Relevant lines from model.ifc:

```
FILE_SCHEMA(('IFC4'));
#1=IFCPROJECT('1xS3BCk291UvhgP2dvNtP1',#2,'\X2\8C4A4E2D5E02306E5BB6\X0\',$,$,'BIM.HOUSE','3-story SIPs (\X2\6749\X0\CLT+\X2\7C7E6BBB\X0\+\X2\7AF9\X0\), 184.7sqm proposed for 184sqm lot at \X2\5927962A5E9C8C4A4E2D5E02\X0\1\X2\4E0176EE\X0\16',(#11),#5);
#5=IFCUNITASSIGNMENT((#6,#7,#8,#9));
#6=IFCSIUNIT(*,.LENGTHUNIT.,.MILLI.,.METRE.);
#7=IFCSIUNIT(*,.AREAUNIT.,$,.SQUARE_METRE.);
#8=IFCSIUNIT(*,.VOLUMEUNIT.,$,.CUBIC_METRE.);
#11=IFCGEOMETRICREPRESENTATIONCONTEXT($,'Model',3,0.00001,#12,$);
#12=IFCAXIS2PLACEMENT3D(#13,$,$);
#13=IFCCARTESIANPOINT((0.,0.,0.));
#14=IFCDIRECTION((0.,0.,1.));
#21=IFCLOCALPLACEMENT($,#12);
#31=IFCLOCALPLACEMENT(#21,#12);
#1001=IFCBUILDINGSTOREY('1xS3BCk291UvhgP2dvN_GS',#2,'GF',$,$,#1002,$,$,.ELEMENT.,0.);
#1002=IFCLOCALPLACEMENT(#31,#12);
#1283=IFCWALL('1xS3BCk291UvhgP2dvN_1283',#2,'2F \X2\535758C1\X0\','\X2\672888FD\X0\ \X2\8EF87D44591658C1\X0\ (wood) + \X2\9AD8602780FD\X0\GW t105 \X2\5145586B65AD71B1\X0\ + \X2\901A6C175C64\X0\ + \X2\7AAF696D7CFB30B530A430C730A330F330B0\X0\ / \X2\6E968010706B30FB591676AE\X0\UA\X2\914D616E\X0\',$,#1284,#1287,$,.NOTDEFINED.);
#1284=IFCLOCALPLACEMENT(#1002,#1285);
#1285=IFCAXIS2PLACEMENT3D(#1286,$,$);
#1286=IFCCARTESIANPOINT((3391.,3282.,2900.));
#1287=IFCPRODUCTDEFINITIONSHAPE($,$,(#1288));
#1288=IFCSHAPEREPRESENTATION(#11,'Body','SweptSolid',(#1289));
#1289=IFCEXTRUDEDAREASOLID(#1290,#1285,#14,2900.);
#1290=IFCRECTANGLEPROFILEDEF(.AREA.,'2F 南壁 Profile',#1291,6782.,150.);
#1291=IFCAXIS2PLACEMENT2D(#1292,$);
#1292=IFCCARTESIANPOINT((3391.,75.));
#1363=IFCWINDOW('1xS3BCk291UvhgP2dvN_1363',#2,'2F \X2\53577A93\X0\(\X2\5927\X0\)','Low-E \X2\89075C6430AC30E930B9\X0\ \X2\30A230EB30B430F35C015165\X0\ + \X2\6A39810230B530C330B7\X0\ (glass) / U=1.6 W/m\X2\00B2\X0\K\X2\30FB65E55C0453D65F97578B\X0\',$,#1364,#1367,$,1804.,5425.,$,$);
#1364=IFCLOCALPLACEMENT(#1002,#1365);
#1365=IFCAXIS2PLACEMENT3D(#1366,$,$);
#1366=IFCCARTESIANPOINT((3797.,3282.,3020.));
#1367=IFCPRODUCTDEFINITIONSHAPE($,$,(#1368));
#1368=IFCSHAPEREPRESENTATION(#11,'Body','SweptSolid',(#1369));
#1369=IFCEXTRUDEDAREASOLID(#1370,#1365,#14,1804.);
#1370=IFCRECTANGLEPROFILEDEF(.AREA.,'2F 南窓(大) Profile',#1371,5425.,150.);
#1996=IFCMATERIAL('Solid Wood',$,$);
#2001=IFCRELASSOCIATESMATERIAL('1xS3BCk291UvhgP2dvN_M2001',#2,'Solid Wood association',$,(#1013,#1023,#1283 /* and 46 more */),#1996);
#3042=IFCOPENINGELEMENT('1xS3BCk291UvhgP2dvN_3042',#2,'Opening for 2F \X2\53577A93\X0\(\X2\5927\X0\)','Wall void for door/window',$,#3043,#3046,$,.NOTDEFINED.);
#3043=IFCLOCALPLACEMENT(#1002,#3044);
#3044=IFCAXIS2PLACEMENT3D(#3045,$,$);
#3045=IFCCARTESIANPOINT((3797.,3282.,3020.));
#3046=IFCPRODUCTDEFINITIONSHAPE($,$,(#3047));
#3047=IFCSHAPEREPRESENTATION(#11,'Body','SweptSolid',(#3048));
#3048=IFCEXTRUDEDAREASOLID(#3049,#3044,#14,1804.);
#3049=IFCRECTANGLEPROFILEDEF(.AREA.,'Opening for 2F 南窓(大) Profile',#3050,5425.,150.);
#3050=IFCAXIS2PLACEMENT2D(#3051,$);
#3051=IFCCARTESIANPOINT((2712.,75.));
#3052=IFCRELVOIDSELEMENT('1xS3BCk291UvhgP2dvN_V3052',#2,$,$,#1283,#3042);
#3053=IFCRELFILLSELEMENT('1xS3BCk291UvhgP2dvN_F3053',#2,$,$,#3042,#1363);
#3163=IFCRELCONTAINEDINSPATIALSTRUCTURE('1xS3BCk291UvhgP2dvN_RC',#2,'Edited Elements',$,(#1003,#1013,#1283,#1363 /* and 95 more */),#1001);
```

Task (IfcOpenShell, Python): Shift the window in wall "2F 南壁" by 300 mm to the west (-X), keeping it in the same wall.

```python
import ifcopenshell
import ifcopenshell.api.geometry
import ifcopenshell.util.placement
import ifcopenshell.util.unit

model = ifcopenshell.open("model.ifc")
unit_scale = ifcopenshell.util.unit.calculate_unit_scale(model)

window = model.by_guid("1xS3BCk291UvhgP2dvN_1363")
opening = window.FillsVoids[0].RelatingOpeningElement
wall = opening.VoidsElements[0].RelatingBuildingElement

wall_matrix = ifcopenshell.util.placement.get_local_placement(wall.ObjectPlacement)
shift = wall_matrix[:3, 0] * -0.3 / unit_scale
before = ifcopenshell.util.placement.get_local_placement(window.ObjectPlacement)[:3, 3].copy()

# The window is not placed relative to its opening, so move both.
for product in (opening, window):
    matrix = ifcopenshell.util.placement.get_local_placement(product.ObjectPlacement)
    matrix[:3, 3] += shift
    ifcopenshell.api.geometry.edit_object_placement(model, product=product, matrix=matrix, is_si=False)

after = ifcopenshell.util.placement.get_local_placement(window.ObjectPlacement)[:3, 3]
print("window moved by", (after - before).round(3) + 0.0)

model.write("model_edited.ifc")
```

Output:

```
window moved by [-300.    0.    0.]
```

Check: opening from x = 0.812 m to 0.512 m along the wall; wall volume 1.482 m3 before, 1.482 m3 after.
